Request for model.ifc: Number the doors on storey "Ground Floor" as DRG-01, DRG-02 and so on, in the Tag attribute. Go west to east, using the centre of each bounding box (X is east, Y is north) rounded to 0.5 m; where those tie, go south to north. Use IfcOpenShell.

First a look at what the model holds.

```python
import ifcopenshell
import ifcopenshell.util.element
import ifcopenshell.util.placement

model = ifcopenshell.open("model.ifc")
print(model.schema)
storey = next(s for s in model.by_type("IfcBuildingStorey") if s.Name == "Ground Floor")
doors = [e for e in ifcopenshell.util.element.get_decomposition(storey) if e.is_a("IfcDoor")]
for e in sorted(doors, key=lambda e: e.id()):
    origin = ifcopenshell.util.placement.get_local_placement(e.ObjectPlacement)[:3, 3]
    print(e.id(), e.Tag, e.Name, origin.round(2) + 0.0, sep=" | ")
```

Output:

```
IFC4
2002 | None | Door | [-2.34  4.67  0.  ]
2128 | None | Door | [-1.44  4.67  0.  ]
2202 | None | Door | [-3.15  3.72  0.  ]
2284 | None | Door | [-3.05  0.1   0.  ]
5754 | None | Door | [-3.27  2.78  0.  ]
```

```python
import ifcopenshell
import ifcopenshell.geom
import ifcopenshell.util.element
import ifcopenshell.util.shape

model = ifcopenshell.open("model.ifc")
settings = ifcopenshell.geom.settings()
settings.set("use-world-coords", True)


def centre(element):
    shape = ifcopenshell.geom.create_shape(settings, element)
    return ifcopenshell.util.shape.get_bbox_centroid(shape.geometry)


storey = next(s for s in model.by_type("IfcBuildingStorey") if s.Name == "Ground Floor")
doors = [e for e in ifcopenshell.util.element.get_decomposition(storey) if e.is_a("IfcDoor")]

# Insertion points can sit at a corner or the storey origin, so sort by the geometry (in metres).
centres = {e: centre(e) for e in doors}
doors.sort(key=lambda e: (round(centres[e][0] / 0.5), centres[e][1]))

for i, e in enumerate(doors, start=1):
    number = f"DRG-{i:02d}"
    e.Tag = number
    print(e.id(), number)

model.write("model_edited.ifc")
```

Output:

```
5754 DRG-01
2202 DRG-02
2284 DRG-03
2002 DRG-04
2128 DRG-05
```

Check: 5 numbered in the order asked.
